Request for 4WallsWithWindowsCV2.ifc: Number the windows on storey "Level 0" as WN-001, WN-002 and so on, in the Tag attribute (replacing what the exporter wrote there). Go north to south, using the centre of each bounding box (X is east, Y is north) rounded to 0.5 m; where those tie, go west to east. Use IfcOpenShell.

First a look at what the model holds.

```python
import ifcopenshell
import ifcopenshell.util.element
import ifcopenshell.util.placement

model = ifcopenshell.open("4WallsWithWindowsCV2.ifc")
print(model.schema)
storey = next(s for s in model.by_type("IfcBuildingStorey") if s.Name == "Level 0")
windows = [e for e in ifcopenshell.util.element.get_decomposition(storey) if e.is_a("IfcWindow")]
for e in sorted(windows, key=lambda e: e.id()):
    origin = ifcopenshell.util.placement.get_local_placement(e.ObjectPlacement)[:3, 3]
    print(e.id(), e.Tag, e.Name, origin.round(2) + 0.0, sep=" | ")
```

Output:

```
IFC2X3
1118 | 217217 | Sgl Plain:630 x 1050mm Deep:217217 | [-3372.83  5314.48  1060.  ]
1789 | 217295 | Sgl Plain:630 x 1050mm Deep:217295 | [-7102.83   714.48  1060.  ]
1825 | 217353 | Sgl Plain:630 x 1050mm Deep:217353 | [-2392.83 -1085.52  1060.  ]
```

```python
import ifcopenshell
import ifcopenshell.geom
import ifcopenshell.util.element
import ifcopenshell.util.shape

model = ifcopenshell.open("4WallsWithWindowsCV2.ifc")
settings = ifcopenshell.geom.settings()
settings.set("use-world-coords", True)


def centre(element):
    shape = ifcopenshell.geom.create_shape(settings, element)
    return ifcopenshell.util.shape.get_bbox_centroid(shape.geometry)


storey = next(s for s in model.by_type("IfcBuildingStorey") if s.Name == "Level 0")
windows = [e for e in ifcopenshell.util.element.get_decomposition(storey) if e.is_a("IfcWindow")]

# Insertion points can sit at a corner or the storey origin, so sort by the geometry (in metres).
centres = {e: centre(e) for e in windows}
windows.sort(key=lambda e: (-round(centres[e][1] / 0.5), centres[e][0]))

for i, e in enumerate(windows, start=1):
    number = f"WN-0{i:02d}"
    e.Tag = number
    print(e.id(), number)

model.write("4WallsWithWindowsCV2-out.ifc")
```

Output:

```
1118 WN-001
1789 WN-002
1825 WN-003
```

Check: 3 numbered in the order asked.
